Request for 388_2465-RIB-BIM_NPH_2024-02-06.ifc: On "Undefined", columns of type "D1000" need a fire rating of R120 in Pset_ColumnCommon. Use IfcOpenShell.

First a look at what the model holds.

```python
import ifcopenshell
import ifcopenshell.util.element

model = ifcopenshell.open("388_2465-RIB-BIM_NPH_2024-02-06.ifc")
print(model.schema)
storey = next(s for s in model.by_type("IfcBuildingStorey") if s.Name == "Undefined")
columns = [e for e in ifcopenshell.util.element.get_decomposition(storey) if e.is_a("IfcColumn")]
seen = {}
for e in columns:
    element_type = ifcopenshell.util.element.get_type(e)
    key = (element_type.Name if element_type != e and element_type else None, ifcopenshell.util.element.get_pset(e, "Pset_ColumnCommon", "FireRating"))
    seen[key] = seen.get(key, 0) + 1
for (name, value), count in sorted(seen.items(), key=str):
    print(count, "x", name, "|", value)
```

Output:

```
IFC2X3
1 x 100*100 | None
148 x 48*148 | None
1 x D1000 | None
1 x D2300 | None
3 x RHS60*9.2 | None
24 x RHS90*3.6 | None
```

```python
import ifcopenshell
import ifcopenshell.api.pset
import ifcopenshell.util.element

model = ifcopenshell.open("388_2465-RIB-BIM_NPH_2024-02-06.ifc")

storey = next(s for s in model.by_type("IfcBuildingStorey") if s.Name == "Undefined")
columns = [e for e in ifcopenshell.util.element.get_decomposition(storey) if e.is_a("IfcColumn")]

count = 0
for e in columns:
    element_type = ifcopenshell.util.element.get_type(e)
    if element_type in (None, e) or element_type.Name != "D1000":
        continue
    # add_pset returns the element's existing set when there is one.
    pset = ifcopenshell.api.pset.add_pset(model, product=e, name="Pset_ColumnCommon")
    ifcopenshell.api.pset.edit_pset(model, pset=pset, properties={"FireRating": "R120"})
    count += 1

print(count, "columns updated")

model.write("388_2465-RIB-BIM_NPH_2024-02-06_v2.ifc")
```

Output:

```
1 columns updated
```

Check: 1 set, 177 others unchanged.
